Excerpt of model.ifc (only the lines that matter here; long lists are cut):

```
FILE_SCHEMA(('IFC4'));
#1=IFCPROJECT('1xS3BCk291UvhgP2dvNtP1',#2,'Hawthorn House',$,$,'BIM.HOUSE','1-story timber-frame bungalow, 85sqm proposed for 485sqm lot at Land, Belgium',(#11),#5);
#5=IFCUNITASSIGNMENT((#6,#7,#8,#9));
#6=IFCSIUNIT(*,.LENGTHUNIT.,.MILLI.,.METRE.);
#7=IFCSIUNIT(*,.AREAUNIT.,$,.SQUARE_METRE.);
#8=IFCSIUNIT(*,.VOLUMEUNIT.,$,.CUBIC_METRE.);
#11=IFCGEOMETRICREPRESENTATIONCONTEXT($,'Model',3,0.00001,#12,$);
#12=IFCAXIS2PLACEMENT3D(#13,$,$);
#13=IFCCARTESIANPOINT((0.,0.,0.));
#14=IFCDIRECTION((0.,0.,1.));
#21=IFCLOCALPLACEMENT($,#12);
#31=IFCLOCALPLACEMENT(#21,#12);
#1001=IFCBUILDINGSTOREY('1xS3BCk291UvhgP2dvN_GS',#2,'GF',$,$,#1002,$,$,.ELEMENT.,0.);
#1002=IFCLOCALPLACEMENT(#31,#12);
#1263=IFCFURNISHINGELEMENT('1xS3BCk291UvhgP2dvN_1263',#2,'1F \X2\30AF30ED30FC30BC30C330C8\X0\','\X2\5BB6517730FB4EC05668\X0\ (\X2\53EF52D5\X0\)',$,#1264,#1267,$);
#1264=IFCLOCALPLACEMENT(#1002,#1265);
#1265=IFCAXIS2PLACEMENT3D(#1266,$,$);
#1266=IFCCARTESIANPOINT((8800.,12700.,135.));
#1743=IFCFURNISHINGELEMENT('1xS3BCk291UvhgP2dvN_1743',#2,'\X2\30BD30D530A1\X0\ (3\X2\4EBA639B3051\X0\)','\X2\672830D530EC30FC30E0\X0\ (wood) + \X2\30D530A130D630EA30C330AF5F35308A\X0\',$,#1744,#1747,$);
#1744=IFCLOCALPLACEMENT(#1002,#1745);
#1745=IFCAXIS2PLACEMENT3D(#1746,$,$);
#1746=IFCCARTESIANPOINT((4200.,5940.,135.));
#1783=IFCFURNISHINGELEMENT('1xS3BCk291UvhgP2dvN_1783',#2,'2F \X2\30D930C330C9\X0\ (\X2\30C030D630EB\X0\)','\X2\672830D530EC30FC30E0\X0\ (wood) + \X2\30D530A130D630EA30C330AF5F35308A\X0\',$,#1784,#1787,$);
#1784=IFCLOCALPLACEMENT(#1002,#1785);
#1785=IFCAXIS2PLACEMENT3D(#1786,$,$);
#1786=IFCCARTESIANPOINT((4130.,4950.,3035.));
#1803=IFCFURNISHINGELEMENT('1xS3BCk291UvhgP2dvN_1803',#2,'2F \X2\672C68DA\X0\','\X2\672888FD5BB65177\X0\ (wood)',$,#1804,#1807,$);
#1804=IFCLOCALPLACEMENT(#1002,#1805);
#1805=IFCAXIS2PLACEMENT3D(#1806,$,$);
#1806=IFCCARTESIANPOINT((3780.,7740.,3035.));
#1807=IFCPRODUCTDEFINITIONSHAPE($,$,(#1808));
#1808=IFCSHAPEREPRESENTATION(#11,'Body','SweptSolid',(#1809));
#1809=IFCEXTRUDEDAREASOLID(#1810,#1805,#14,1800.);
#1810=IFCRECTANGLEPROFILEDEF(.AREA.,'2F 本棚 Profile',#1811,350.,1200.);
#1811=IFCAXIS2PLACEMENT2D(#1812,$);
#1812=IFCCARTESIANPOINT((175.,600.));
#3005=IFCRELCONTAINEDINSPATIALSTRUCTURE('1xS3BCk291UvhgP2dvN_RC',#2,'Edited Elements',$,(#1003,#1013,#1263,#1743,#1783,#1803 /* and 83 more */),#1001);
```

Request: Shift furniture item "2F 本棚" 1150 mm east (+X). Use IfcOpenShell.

```python
import ifcopenshell
import ifcopenshell.api.geometry
import ifcopenshell.util.placement

model = ifcopenshell.open("model.ifc")

item = model.by_guid("1xS3BCk291UvhgP2dvN_1803")
matrix = ifcopenshell.util.placement.get_local_placement(item.ObjectPlacement)
matrix[0, 3] += 1150.0
ifcopenshell.api.geometry.edit_object_placement(model, product=item, matrix=matrix, is_si=False)

print(ifcopenshell.util.placement.get_local_placement(item.ObjectPlacement).round(3) + 0.0)

model.write("model_rev.ifc")
```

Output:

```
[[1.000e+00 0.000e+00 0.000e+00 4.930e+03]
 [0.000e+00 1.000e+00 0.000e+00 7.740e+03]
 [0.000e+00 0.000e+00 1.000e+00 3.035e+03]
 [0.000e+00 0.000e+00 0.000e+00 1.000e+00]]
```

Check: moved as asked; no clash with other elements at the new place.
